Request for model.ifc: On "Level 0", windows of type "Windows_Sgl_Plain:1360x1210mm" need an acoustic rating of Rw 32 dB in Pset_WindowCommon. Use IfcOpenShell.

First a look at what the model holds.

```python
import ifcopenshell
import ifcopenshell.util.element

model = ifcopenshell.open("model.ifc")
print(model.schema)
storey = next(s for s in model.by_type("IfcBuildingStorey") if s.Name == "Level 0")
windows = [e for e in ifcopenshell.util.element.get_decomposition(storey) if e.is_a("IfcWindow")]
seen = {}
for e in windows:
    element_type = ifcopenshell.util.element.get_type(e)
    key = (element_type.Name if element_type != e and element_type else None, ifcopenshell.util.element.get_pset(e, "Pset_WindowCommon", "AcousticRating"))
    seen[key] = seen.get(key, 0) + 1
for (name, value), count in sorted(seen.items(), key=str):
    print(count, "x", name, "|", value)
```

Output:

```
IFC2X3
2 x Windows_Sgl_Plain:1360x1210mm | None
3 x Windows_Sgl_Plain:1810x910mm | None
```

```python
import ifcopenshell
import ifcopenshell.api.pset
import ifcopenshell.util.element

model = ifcopenshell.open("model.ifc")

storey = next(s for s in model.by_type("IfcBuildingStorey") if s.Name == "Level 0")
windows = [e for e in ifcopenshell.util.element.get_decomposition(storey) if e.is_a("IfcWindow")]

count = 0
for e in windows:
    element_type = ifcopenshell.util.element.get_type(e)
    if element_type in (None, e) or element_type.Name != "Windows_Sgl_Plain:1360x1210mm":
        continue
    # add_pset returns the element's existing set when there is one.
    pset = ifcopenshell.api.pset.add_pset(model, product=e, name="Pset_WindowCommon")
    ifcopenshell.api.pset.edit_pset(model, pset=pset, properties={"AcousticRating": "Rw 32 dB"})
    count += 1

print(count, "windows updated")

model.write("model_rev.ifc")
```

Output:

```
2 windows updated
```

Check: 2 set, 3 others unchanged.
